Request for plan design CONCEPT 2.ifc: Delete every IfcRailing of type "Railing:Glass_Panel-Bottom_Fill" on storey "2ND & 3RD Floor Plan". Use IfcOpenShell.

First a look at what the model holds.

```python
import ifcopenshell
import ifcopenshell.util.element

model = ifcopenshell.open("plan design CONCEPT 2.ifc")
print(model.schema)
storey = next(s for s in model.by_type("IfcBuildingStorey") if s.Name == "2ND & 3RD Floor Plan")
railings = [e for e in ifcopenshell.util.element.get_decomposition(storey) if e.is_a("IfcRailing")]
seen = {}
for e in railings:
    element_type = ifcopenshell.util.element.get_type(e)
    name = element_type.Name if element_type not in (None, e) else None
    seen[name] = seen.get(name, 0) + 1
for name, count in sorted(seen.items(), key=str):
    print(count, "x", name)
```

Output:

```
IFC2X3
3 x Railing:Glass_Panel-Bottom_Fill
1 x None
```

```python
import ifcopenshell
import ifcopenshell.api.root
import ifcopenshell.util.element

model = ifcopenshell.open("plan design CONCEPT 2.ifc")

storey = next(s for s in model.by_type("IfcBuildingStorey") if s.Name == "2ND & 3RD Floor Plan")
railings = [e for e in ifcopenshell.util.element.get_decomposition(storey) if e.is_a("IfcRailing")]
targets = [e for e in railings if (t := ifcopenshell.util.element.get_type(e)) not in (None, e) and t.Name == "Railing:Glass_Panel-Bottom_Fill"]

for e in targets:
    ifcopenshell.api.root.remove_product(model, product=e)
print(len(targets), "removed")

model.write("plan design CONCEPT 2_updated.ifc")
```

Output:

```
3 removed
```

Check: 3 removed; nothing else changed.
